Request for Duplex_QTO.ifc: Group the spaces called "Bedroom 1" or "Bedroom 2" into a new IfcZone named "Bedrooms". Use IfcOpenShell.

First a look at what the model holds.

```python
import ifcopenshell

model = ifcopenshell.open("Duplex_QTO.ifc")
print(model.schema)
seen = {}
for space in model.by_type("IfcSpace"):
    seen[space.LongName] = seen.get(space.LongName, 0) + 1
for name, count in sorted(seen.items(), key=str):
    print(count, "x", name)
print("zones:", [z.Name for z in model.by_type("IfcZone")][:20])
```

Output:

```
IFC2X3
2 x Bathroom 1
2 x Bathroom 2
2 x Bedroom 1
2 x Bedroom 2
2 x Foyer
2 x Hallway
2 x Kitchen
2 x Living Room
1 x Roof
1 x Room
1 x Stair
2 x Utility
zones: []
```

```python
import ifcopenshell
import ifcopenshell.api.group
import ifcopenshell.api.root

model = ifcopenshell.open("Duplex_QTO.ifc")

names = {"Bedroom 1", "Bedroom 2"}
spaces = [s for s in model.by_type("IfcSpace") if s.LongName in names]

zone = ifcopenshell.api.root.create_entity(model, ifc_class="IfcZone", name="Bedrooms")
ifcopenshell.api.group.assign_group(model, products=spaces, group=zone)
print(len(spaces), "spaces in", zone.Name)

model.write("Duplex_QTO_edited.ifc")
```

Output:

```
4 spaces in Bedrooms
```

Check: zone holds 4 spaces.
